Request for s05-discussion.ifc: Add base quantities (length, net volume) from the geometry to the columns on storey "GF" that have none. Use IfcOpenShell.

First a look at what the model holds.

```python
import ifcopenshell
import ifcopenshell.util.element
import ifcopenshell.util.unit

model = ifcopenshell.open("s05-discussion.ifc")
print(model.schema)
for unit_type in ("LENGTHUNIT", "AREAUNIT", "VOLUMEUNIT"):
    print(unit_type, ifcopenshell.util.unit.calculate_unit_scale(model, unit_type))
storey = next(s for s in model.by_type("IfcBuildingStorey") if s.Name == "GF")
columns = [e for e in ifcopenshell.util.element.get_decomposition(storey) if e.is_a("IfcColumn")]
for e in sorted(columns, key=lambda e: e.id()):
    print(e.id(), e.is_a(), e.Name, list(ifcopenshell.util.element.get_psets(e, qtos_only=True)), sep=" | ")
```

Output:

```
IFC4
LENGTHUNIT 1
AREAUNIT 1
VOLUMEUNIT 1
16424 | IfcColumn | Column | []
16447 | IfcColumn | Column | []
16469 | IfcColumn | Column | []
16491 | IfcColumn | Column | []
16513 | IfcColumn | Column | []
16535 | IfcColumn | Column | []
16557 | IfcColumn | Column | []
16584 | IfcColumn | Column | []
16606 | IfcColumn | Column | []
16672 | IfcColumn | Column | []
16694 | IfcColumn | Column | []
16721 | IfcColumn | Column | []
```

```python
import ifcopenshell
import ifcopenshell.api.pset
import ifcopenshell.geom
import ifcopenshell.util.element
import ifcopenshell.util.shape
import ifcopenshell.util.unit

model = ifcopenshell.open("s05-discussion.ifc")
unit_scale = ifcopenshell.util.unit.calculate_unit_scale(model)
volume_scale = ifcopenshell.util.unit.calculate_unit_scale(model, "VOLUMEUNIT")
settings = ifcopenshell.geom.settings()

storey = next(s for s in model.by_type("IfcBuildingStorey") if s.Name == "GF")
columns = [e for e in ifcopenshell.util.element.get_decomposition(storey) if e.is_a("IfcColumn")]

for e in sorted(columns, key=lambda e: e.id()):
    if ifcopenshell.util.element.get_psets(e, qtos_only=True, should_inherit=False):
        continue
    # Geometry comes back in metres, in the element's own axes.
    shape = ifcopenshell.geom.create_shape(settings, e)
    values = {
        "Length": ifcopenshell.util.shape.get_z(shape.geometry) / unit_scale,
        "NetVolume": ifcopenshell.util.shape.get_volume(shape.geometry) / volume_scale,
    }
    qto = ifcopenshell.api.pset.add_qto(model, product=e, name="Qto_ColumnBaseQuantities")
    ifcopenshell.api.pset.edit_qto(model, qto=qto, properties=values)
    print(e.id(), {k: round(v, 3) for k, v in values.items()})

model.write("s05-discussion_edited.ifc")
```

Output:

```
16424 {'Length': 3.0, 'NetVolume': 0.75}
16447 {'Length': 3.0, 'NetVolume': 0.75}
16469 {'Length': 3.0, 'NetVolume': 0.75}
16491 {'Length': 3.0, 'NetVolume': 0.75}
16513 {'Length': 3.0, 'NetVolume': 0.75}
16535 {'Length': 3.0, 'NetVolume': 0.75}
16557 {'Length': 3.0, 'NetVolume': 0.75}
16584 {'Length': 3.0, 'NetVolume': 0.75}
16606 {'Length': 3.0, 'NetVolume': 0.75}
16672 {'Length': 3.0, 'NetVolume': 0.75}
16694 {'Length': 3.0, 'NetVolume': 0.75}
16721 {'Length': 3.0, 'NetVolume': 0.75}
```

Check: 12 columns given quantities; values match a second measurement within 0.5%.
